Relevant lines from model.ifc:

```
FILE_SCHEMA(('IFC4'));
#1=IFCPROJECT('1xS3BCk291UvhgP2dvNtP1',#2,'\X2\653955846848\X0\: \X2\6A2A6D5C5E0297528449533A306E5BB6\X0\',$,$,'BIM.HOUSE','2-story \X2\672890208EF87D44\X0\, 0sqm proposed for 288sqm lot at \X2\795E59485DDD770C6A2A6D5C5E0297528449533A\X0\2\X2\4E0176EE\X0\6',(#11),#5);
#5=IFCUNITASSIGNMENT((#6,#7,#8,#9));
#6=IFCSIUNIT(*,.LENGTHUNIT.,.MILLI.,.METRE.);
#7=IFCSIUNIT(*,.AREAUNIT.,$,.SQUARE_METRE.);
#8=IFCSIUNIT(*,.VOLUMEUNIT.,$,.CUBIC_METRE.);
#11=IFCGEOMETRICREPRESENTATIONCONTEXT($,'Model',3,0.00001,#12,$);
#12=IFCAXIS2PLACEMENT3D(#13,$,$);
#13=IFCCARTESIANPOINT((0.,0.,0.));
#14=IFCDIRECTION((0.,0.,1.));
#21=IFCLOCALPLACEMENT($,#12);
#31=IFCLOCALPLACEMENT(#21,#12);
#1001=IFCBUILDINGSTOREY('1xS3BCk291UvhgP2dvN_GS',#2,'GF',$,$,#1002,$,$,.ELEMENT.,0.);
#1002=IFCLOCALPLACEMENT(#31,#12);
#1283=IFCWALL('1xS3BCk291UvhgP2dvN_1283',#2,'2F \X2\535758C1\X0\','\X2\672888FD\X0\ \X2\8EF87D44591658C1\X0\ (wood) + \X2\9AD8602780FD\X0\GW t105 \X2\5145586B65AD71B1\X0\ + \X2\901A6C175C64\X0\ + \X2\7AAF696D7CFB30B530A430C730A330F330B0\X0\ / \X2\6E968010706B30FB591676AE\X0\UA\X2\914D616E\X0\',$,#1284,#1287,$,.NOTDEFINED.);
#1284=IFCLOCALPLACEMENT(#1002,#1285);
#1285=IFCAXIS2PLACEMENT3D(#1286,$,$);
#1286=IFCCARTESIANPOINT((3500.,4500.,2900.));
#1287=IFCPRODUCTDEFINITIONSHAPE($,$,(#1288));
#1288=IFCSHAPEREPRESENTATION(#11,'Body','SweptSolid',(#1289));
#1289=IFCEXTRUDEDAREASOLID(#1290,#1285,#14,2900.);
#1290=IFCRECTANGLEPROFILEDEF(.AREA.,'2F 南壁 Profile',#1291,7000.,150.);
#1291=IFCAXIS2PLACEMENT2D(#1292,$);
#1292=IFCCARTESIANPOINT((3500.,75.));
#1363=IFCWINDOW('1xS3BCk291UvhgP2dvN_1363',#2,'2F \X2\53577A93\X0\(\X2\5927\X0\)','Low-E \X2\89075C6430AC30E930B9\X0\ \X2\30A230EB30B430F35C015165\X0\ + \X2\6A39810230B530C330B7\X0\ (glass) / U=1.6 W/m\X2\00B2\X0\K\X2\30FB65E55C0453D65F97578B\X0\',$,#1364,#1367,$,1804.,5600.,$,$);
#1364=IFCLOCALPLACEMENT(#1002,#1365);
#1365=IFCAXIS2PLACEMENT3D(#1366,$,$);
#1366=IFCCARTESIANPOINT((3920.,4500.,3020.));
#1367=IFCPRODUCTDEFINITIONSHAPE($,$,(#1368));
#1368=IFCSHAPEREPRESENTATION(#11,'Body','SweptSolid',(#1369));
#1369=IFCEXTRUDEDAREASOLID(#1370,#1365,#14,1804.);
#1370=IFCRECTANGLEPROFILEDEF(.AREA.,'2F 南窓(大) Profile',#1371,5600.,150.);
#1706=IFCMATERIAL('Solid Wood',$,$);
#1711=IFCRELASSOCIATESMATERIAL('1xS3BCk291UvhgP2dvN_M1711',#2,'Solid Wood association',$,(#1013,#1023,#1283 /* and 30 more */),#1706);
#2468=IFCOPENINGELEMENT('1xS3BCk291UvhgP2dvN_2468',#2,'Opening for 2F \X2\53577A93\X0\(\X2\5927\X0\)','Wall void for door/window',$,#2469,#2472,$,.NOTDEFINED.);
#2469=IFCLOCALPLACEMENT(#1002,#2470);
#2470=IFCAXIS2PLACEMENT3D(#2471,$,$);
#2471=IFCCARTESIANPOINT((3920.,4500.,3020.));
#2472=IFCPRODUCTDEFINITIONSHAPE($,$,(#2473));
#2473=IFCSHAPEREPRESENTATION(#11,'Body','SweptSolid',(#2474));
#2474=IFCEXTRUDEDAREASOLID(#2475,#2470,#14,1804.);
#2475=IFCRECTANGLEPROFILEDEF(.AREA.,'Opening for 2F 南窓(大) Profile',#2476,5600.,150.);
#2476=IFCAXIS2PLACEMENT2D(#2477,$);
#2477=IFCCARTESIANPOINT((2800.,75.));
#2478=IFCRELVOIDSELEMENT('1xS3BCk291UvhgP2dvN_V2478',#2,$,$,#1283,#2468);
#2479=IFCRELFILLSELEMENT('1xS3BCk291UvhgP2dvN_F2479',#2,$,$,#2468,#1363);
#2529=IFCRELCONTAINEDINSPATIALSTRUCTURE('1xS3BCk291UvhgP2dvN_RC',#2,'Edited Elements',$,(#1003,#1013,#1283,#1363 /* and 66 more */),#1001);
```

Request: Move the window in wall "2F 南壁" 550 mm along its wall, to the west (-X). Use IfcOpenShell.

```python
import ifcopenshell
import ifcopenshell.api.geometry
import ifcopenshell.util.placement
import ifcopenshell.util.unit

model = ifcopenshell.open("model.ifc")
unit_scale = ifcopenshell.util.unit.calculate_unit_scale(model)

window = model.by_guid("1xS3BCk291UvhgP2dvN_1363")
opening = window.FillsVoids[0].RelatingOpeningElement
wall = opening.VoidsElements[0].RelatingBuildingElement

wall_matrix = ifcopenshell.util.placement.get_local_placement(wall.ObjectPlacement)
shift = wall_matrix[:3, 0] * -0.55 / unit_scale
before = ifcopenshell.util.placement.get_local_placement(window.ObjectPlacement)[:3, 3].copy()

# The window is not placed relative to its opening, so move both.
for product in (opening, window):
    matrix = ifcopenshell.util.placement.get_local_placement(product.ObjectPlacement)
    matrix[:3, 3] += shift
    ifcopenshell.api.geometry.edit_object_placement(model, product=product, matrix=matrix, is_si=False)

after = ifcopenshell.util.placement.get_local_placement(window.ObjectPlacement)[:3, 3]
print("window moved by", (after - before).round(3) + 0.0)

model.write("model-out.ifc")
```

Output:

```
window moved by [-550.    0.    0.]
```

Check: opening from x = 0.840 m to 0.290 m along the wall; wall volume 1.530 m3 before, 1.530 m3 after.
